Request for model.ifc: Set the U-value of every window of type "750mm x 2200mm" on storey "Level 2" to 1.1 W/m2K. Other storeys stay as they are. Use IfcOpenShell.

First a look at what the model holds.

```python
import ifcopenshell
import ifcopenshell.util.element

model = ifcopenshell.open("model.ifc")
print(model.schema)
storey = next(s for s in model.by_type("IfcBuildingStorey") if s.Name == "Level 2")
windows = [e for e in ifcopenshell.util.element.get_decomposition(storey) if e.is_a("IfcWindow")]
seen = {}
for e in windows:
    element_type = ifcopenshell.util.element.get_type(e)
    key = (element_type.Name if element_type != e and element_type else None, ifcopenshell.util.element.get_pset(e, "Pset_WindowCommon", "ThermalTransmittance"))
    seen[key] = seen.get(key, 0) + 1
for (name, value), count in sorted(seen.items(), key=str):
    print(count, "x", name, "|", value)
```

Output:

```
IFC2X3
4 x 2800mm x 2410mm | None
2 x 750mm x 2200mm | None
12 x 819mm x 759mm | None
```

```python
import ifcopenshell
import ifcopenshell.api.pset
import ifcopenshell.util.element

model = ifcopenshell.open("model.ifc")

storey = next(s for s in model.by_type("IfcBuildingStorey") if s.Name == "Level 2")
windows = [e for e in ifcopenshell.util.element.get_decomposition(storey) if e.is_a("IfcWindow")]

count = 0
for e in windows:
    element_type = ifcopenshell.util.element.get_type(e)
    if element_type in (None, e) or element_type.Name != "750mm x 2200mm":
        continue
    # add_pset returns the element's existing set when there is one.
    pset = ifcopenshell.api.pset.add_pset(model, product=e, name="Pset_WindowCommon")
    ifcopenshell.api.pset.edit_pset(model, pset=pset, properties={"ThermalTransmittance": 1.1})
    count += 1

print(count, "windows updated")

model.write("model_rev.ifc")
```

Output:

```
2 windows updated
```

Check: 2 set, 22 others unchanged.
